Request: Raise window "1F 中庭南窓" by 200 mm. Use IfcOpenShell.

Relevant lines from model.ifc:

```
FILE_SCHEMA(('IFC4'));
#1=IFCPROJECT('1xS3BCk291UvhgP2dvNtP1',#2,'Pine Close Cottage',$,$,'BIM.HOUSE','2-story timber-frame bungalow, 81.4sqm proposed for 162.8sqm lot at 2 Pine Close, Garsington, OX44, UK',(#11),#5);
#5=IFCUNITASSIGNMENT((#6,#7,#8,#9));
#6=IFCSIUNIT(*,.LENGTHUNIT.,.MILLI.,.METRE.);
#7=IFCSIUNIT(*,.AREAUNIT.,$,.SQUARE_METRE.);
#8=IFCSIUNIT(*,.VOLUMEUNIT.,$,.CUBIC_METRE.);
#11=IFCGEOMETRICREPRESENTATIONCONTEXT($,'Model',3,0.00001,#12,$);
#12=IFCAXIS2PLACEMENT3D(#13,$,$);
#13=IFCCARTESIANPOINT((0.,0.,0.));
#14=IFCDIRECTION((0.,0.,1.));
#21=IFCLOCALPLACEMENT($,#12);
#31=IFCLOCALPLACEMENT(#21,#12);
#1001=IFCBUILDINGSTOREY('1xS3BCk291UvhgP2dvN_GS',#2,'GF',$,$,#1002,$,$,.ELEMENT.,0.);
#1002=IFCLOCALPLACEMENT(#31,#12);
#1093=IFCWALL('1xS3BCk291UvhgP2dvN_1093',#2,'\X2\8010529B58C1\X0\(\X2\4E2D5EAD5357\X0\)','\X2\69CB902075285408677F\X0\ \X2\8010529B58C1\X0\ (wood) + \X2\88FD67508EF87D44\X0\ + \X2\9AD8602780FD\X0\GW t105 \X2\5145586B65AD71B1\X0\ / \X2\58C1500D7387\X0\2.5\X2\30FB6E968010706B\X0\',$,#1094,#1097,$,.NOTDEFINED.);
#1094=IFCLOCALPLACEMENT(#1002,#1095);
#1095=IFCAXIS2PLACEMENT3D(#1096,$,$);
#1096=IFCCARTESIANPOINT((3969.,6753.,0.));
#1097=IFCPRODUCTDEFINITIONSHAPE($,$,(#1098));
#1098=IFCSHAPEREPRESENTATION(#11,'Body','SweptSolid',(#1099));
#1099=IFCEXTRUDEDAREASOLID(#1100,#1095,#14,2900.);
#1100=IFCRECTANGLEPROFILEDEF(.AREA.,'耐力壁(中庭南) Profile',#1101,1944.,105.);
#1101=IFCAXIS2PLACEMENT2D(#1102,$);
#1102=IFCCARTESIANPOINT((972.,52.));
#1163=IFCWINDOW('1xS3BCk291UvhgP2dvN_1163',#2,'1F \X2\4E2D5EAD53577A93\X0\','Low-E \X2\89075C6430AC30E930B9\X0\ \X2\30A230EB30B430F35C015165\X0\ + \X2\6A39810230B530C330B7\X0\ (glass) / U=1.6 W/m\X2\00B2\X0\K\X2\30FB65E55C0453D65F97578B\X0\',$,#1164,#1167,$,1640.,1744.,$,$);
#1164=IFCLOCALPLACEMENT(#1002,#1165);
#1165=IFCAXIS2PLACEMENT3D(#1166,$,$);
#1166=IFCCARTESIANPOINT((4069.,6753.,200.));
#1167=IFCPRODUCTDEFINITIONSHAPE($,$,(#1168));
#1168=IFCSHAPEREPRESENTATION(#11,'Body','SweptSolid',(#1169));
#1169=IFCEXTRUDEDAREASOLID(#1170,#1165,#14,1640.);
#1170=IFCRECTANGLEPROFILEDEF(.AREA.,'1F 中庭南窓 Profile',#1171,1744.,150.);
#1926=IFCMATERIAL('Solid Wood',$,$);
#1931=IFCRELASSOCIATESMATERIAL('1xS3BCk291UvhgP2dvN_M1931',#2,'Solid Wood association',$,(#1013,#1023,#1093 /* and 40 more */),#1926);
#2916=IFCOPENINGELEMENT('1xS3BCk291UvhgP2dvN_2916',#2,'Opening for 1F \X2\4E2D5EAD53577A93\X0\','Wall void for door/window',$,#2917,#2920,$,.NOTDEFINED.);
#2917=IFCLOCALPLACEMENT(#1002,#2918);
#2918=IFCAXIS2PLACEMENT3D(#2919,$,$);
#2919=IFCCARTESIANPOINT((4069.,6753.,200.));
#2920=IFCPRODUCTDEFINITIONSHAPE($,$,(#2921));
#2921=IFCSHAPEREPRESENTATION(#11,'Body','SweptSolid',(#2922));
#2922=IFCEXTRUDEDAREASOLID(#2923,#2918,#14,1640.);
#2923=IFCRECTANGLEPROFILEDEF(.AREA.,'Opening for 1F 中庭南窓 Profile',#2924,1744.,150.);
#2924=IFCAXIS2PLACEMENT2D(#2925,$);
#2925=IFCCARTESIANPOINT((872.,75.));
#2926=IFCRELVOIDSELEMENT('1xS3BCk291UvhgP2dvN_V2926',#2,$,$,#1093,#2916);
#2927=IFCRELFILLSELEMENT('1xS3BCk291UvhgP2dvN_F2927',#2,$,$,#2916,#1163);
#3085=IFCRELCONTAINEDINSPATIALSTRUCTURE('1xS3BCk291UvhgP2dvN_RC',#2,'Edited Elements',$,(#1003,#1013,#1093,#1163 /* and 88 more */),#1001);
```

```python
import numpy as np
import ifcopenshell
import ifcopenshell.api.geometry
import ifcopenshell.util.placement
import ifcopenshell.util.unit

model = ifcopenshell.open("model.ifc")
unit_scale = ifcopenshell.util.unit.calculate_unit_scale(model)

window = model.by_guid("1xS3BCk291UvhgP2dvN_1163")
opening = window.FillsVoids[0].RelatingOpeningElement
dz = 0.2 / unit_scale

shift = np.array([0.0, 0.0, dz])
# The window is not placed relative to its opening, so move both.
for product in (opening, window):
    matrix = ifcopenshell.util.placement.get_local_placement(product.ObjectPlacement)
    matrix[:3, 3] += shift
    ifcopenshell.api.geometry.edit_object_placement(model, product=product, matrix=matrix, is_si=False)

print(f"moved by {dz * unit_scale:+.3f} m")

model.write("model_v2.ifc")
```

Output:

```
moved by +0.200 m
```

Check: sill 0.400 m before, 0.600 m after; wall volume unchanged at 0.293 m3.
